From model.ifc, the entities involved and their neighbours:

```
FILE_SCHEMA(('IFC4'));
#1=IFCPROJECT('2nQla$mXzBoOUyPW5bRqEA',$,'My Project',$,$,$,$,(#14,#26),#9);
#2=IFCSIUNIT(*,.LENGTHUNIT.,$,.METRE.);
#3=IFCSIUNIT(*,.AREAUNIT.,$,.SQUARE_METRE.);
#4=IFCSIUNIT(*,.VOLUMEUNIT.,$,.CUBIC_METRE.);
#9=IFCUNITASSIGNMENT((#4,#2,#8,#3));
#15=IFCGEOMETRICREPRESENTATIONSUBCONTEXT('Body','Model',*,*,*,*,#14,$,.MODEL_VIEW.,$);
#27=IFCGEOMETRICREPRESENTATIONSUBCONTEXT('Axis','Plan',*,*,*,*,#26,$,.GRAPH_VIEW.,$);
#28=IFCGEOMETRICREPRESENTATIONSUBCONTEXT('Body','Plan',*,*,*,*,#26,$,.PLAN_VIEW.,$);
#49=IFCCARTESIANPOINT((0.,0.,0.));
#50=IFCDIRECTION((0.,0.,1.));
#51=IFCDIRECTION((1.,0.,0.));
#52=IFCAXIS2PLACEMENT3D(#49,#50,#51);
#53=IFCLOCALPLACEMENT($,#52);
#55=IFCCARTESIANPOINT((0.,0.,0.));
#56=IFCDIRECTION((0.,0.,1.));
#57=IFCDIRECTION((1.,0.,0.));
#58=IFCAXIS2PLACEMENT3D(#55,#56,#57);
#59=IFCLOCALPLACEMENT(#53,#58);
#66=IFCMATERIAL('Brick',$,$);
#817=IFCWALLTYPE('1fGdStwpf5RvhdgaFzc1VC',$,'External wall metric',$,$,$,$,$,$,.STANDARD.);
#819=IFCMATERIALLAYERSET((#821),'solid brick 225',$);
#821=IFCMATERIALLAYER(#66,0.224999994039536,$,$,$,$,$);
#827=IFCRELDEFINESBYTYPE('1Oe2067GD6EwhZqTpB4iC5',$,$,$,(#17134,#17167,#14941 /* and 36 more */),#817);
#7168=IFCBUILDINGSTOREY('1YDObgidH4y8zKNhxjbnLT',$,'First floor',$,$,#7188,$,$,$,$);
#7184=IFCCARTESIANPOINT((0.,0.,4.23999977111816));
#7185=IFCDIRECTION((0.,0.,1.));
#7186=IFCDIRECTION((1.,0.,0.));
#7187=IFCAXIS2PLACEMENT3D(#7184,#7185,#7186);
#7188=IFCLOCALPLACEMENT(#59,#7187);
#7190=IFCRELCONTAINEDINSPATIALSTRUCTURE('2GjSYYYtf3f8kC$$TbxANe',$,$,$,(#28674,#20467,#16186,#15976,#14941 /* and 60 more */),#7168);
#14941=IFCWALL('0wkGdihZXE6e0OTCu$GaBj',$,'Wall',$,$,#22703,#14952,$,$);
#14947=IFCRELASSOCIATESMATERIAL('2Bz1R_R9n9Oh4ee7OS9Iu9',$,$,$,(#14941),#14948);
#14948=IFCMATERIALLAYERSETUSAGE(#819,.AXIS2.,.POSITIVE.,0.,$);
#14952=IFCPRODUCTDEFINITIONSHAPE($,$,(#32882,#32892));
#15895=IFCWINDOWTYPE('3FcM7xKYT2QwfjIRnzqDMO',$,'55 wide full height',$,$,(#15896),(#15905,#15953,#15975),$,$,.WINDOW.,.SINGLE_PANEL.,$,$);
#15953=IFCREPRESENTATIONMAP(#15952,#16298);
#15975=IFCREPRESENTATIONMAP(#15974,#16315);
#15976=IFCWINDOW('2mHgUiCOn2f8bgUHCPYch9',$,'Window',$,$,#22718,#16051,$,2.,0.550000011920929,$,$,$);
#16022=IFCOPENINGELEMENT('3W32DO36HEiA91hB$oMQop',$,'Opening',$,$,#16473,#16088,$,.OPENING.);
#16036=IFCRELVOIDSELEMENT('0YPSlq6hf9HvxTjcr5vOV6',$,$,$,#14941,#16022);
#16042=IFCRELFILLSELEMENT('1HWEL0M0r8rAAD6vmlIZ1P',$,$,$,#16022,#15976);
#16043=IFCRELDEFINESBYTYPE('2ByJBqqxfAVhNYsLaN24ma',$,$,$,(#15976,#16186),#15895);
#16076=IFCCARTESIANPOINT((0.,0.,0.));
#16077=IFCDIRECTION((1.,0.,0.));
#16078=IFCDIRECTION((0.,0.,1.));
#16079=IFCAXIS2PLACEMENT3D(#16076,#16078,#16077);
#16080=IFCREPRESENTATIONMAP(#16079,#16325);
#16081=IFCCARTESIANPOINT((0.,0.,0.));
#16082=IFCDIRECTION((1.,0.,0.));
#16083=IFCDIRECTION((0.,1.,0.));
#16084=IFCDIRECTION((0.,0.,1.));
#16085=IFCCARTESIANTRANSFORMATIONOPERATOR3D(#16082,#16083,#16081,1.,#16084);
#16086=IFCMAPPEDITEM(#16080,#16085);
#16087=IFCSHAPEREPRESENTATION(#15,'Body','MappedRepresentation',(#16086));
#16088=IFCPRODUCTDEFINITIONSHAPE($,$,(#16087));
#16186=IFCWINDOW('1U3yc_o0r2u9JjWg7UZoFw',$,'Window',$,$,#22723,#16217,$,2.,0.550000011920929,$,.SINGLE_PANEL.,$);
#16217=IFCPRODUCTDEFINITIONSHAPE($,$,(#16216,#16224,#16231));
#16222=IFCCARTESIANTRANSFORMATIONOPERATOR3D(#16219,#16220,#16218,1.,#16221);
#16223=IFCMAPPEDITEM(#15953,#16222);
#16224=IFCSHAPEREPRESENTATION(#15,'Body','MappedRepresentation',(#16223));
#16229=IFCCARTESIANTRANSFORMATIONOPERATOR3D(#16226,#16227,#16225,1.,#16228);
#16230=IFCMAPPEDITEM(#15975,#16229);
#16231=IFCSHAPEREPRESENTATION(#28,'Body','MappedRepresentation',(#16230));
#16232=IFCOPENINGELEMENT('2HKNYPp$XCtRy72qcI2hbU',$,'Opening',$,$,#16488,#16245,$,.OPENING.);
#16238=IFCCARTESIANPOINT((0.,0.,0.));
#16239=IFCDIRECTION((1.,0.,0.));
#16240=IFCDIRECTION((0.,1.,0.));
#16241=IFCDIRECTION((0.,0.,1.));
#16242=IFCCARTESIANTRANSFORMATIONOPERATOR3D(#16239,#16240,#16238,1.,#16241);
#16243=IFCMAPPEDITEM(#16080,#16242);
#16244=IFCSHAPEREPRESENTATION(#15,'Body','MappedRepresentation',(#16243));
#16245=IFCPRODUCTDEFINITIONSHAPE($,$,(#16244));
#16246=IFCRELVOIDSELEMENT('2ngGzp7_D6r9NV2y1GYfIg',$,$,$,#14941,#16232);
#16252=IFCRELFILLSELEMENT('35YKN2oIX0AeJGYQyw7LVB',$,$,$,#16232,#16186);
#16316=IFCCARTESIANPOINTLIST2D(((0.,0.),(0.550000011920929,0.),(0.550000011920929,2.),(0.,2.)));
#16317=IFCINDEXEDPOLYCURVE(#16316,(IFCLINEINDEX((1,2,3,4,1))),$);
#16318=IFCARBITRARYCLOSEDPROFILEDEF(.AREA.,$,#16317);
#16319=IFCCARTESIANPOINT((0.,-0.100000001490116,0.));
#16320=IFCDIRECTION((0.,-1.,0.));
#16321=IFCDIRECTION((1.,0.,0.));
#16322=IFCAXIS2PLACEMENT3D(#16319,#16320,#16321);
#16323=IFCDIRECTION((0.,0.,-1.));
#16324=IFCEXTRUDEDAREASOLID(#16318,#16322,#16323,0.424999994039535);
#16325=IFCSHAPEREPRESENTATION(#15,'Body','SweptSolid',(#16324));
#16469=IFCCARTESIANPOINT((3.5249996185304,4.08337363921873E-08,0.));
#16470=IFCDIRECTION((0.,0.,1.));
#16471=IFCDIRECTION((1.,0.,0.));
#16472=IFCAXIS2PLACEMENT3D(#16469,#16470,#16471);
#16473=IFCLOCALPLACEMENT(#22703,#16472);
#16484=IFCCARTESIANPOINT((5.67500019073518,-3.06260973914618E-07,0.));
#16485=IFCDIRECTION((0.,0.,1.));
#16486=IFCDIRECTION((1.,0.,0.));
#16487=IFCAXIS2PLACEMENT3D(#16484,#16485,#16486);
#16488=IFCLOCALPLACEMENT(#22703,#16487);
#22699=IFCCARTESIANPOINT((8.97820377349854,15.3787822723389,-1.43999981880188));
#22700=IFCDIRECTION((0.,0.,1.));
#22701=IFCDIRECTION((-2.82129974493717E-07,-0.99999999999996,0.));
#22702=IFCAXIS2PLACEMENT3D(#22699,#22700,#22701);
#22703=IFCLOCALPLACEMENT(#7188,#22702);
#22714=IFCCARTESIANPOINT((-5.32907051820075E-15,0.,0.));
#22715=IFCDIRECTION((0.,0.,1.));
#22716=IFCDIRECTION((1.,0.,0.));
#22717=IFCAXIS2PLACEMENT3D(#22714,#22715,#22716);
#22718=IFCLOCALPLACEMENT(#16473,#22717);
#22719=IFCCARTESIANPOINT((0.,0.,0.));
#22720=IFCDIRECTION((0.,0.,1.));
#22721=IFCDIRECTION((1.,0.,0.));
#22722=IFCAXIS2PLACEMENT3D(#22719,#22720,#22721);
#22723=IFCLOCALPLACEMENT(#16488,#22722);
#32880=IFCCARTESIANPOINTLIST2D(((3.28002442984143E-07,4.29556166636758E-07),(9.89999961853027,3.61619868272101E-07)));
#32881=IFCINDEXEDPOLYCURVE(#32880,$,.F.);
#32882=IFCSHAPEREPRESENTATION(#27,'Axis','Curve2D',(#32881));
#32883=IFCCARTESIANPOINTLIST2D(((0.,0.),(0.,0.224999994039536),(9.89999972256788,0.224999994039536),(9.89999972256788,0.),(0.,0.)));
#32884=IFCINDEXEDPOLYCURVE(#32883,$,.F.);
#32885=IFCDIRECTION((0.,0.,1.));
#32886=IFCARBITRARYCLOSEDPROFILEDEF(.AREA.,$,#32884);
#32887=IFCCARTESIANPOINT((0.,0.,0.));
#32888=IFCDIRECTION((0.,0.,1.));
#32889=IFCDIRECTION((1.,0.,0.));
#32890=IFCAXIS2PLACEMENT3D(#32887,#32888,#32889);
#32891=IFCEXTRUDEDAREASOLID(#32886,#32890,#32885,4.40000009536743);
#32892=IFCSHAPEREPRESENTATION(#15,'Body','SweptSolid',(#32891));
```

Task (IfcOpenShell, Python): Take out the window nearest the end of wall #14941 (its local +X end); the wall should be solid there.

```python
import ifcopenshell
import ifcopenshell.api.feature
import ifcopenshell.api.root
import ifcopenshell.geom
import ifcopenshell.util.shape

model = ifcopenshell.open("model.ifc")
settings = ifcopenshell.geom.settings()


def volume(element):
    """Net volume in cubic metres, openings subtracted."""
    shape = ifcopenshell.geom.create_shape(settings, element)
    return ifcopenshell.util.shape.get_volume(shape.geometry)


window = model.by_id(16186)
opening = window.FillsVoids[0].RelatingOpeningElement
wall = opening.VoidsElements[0].RelatingBuildingElement
before = volume(wall)

ifcopenshell.api.root.remove_product(model, product=window)
ifcopenshell.api.feature.remove_feature(model, feature=opening)

after = volume(wall)

print(f"wall volume {before:.3f} -> {after:.3f} m3")

model.write("model_updated.ifc")
```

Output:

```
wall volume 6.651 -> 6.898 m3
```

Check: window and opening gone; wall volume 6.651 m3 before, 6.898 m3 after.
